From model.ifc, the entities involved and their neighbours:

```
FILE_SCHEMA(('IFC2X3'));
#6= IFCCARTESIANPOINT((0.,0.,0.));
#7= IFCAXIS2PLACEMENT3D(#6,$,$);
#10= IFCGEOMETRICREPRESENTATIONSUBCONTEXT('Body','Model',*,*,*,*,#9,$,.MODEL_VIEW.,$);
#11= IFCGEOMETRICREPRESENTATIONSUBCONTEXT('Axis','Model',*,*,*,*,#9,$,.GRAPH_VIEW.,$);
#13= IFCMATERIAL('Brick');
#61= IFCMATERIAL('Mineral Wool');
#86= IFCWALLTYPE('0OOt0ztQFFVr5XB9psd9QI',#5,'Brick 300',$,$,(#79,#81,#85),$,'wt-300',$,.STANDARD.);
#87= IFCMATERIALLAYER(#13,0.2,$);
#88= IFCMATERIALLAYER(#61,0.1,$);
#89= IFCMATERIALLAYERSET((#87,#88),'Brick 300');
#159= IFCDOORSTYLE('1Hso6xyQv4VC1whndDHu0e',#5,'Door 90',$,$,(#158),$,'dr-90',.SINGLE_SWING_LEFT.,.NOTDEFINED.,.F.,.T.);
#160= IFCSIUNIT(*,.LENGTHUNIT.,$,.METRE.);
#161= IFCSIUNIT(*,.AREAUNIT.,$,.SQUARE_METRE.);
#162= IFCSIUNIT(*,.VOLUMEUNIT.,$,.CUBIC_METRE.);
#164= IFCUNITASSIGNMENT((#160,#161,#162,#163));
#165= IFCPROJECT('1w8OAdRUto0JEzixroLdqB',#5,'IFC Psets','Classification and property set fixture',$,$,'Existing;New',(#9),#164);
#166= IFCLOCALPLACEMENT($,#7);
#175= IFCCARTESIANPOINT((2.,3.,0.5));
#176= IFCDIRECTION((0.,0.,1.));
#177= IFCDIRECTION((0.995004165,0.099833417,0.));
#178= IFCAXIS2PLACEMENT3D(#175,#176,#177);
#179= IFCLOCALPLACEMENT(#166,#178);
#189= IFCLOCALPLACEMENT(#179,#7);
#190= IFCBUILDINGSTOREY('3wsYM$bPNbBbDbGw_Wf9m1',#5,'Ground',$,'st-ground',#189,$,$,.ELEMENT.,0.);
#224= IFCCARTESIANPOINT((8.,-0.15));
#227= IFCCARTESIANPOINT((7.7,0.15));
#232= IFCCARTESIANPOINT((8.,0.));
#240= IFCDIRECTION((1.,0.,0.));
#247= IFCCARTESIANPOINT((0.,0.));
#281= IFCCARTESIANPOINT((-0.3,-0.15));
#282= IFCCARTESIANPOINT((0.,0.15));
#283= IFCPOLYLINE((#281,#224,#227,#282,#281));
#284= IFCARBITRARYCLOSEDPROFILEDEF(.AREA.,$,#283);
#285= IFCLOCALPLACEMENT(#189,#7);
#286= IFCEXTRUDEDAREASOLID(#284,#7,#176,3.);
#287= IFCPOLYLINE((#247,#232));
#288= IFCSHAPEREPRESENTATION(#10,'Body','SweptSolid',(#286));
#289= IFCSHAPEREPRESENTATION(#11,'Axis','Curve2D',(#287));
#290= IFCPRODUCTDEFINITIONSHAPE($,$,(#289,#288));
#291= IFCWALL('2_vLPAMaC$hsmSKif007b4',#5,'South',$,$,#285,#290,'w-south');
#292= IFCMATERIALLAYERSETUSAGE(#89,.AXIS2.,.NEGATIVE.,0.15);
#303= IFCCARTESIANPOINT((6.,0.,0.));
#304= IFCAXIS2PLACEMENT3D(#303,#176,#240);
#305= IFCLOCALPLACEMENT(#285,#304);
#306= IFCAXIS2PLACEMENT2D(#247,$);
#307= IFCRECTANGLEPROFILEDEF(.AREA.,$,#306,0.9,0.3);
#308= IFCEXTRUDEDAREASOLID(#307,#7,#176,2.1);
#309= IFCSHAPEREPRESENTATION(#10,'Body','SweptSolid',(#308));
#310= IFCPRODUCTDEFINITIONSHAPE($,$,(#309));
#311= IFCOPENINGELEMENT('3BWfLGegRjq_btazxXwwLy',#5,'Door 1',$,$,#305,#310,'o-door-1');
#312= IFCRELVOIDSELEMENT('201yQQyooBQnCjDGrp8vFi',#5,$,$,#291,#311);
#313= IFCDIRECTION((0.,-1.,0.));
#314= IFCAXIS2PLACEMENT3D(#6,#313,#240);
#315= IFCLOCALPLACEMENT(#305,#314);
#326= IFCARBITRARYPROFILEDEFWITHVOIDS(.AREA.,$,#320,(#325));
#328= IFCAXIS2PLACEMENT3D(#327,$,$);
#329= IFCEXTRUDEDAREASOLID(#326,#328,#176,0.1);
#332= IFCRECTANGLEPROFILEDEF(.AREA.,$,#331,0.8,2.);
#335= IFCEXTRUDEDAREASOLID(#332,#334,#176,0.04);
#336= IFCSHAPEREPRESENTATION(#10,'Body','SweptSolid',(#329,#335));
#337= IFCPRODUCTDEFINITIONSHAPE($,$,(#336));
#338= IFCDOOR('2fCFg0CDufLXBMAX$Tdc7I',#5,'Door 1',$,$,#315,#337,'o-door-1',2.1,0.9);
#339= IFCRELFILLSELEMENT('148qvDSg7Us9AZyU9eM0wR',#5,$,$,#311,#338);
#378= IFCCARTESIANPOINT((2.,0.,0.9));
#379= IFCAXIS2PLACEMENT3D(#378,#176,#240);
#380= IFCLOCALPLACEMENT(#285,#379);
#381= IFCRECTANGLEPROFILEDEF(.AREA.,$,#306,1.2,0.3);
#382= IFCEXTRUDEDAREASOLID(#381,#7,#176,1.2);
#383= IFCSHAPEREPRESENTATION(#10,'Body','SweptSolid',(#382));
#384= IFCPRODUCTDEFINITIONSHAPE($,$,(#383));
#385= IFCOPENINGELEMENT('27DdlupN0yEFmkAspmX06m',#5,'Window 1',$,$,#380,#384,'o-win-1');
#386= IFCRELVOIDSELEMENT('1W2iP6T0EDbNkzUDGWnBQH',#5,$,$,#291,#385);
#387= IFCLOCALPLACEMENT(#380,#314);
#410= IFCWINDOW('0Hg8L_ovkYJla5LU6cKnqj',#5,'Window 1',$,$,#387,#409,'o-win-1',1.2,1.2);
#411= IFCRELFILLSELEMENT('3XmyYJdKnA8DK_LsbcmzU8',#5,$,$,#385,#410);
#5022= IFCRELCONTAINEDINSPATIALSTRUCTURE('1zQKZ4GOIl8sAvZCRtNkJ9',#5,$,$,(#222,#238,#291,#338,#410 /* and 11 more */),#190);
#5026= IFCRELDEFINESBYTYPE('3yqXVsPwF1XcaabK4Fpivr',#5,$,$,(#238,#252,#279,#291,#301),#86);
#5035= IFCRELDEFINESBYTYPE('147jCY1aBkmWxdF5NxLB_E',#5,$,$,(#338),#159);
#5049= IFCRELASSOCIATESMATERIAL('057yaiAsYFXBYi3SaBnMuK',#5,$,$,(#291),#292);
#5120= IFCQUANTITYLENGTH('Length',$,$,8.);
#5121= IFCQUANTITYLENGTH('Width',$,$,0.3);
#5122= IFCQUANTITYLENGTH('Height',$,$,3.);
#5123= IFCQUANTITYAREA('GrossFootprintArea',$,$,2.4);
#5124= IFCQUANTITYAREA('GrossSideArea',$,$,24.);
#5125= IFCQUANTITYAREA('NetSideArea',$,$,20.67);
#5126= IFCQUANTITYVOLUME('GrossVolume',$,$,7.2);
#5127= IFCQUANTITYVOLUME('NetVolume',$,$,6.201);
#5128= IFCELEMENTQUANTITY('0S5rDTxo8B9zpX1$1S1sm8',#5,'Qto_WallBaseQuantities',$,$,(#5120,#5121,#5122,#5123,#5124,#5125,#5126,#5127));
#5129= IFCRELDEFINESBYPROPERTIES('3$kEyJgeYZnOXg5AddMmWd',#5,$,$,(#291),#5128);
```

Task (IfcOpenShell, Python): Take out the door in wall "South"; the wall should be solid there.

```python
import ifcopenshell
import ifcopenshell.api.feature
import ifcopenshell.api.pset
import ifcopenshell.api.root
import ifcopenshell.geom
import ifcopenshell.util.element
import ifcopenshell.util.shape
import ifcopenshell.util.unit

model = ifcopenshell.open("model.ifc")
area_scale = ifcopenshell.util.unit.calculate_unit_scale(model, "AREAUNIT")
volume_scale = ifcopenshell.util.unit.calculate_unit_scale(model, "VOLUMEUNIT")
settings = ifcopenshell.geom.settings()


def volume(element):
    """Net volume in cubic metres, openings subtracted."""
    shape = ifcopenshell.geom.create_shape(settings, element)
    return ifcopenshell.util.shape.get_volume(shape.geometry)


door = model.by_id(338)
opening = door.FillsVoids[0].RelatingOpeningElement
wall = opening.VoidsElements[0].RelatingBuildingElement
before = volume(wall)

ifcopenshell.api.root.remove_product(model, product=door)
ifcopenshell.api.feature.remove_feature(model, feature=opening)

after = volume(wall)
thickness = 0.3  # wall thickness in metres

# Update the wall's stored quantities.
qto = model.by_id(ifcopenshell.util.element.get_pset(wall, "Qto_WallBaseQuantities", should_inherit=False)["id"])
ifcopenshell.api.pset.edit_qto(model, qto=qto, properties={
    "NetSideArea": after / thickness / area_scale,
    "NetVolume": after / volume_scale,
})

print(f"wall volume {before:.3f} -> {after:.3f} m3")

model.write("model-out.ifc")
```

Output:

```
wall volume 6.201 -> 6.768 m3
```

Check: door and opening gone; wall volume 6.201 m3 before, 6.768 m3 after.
